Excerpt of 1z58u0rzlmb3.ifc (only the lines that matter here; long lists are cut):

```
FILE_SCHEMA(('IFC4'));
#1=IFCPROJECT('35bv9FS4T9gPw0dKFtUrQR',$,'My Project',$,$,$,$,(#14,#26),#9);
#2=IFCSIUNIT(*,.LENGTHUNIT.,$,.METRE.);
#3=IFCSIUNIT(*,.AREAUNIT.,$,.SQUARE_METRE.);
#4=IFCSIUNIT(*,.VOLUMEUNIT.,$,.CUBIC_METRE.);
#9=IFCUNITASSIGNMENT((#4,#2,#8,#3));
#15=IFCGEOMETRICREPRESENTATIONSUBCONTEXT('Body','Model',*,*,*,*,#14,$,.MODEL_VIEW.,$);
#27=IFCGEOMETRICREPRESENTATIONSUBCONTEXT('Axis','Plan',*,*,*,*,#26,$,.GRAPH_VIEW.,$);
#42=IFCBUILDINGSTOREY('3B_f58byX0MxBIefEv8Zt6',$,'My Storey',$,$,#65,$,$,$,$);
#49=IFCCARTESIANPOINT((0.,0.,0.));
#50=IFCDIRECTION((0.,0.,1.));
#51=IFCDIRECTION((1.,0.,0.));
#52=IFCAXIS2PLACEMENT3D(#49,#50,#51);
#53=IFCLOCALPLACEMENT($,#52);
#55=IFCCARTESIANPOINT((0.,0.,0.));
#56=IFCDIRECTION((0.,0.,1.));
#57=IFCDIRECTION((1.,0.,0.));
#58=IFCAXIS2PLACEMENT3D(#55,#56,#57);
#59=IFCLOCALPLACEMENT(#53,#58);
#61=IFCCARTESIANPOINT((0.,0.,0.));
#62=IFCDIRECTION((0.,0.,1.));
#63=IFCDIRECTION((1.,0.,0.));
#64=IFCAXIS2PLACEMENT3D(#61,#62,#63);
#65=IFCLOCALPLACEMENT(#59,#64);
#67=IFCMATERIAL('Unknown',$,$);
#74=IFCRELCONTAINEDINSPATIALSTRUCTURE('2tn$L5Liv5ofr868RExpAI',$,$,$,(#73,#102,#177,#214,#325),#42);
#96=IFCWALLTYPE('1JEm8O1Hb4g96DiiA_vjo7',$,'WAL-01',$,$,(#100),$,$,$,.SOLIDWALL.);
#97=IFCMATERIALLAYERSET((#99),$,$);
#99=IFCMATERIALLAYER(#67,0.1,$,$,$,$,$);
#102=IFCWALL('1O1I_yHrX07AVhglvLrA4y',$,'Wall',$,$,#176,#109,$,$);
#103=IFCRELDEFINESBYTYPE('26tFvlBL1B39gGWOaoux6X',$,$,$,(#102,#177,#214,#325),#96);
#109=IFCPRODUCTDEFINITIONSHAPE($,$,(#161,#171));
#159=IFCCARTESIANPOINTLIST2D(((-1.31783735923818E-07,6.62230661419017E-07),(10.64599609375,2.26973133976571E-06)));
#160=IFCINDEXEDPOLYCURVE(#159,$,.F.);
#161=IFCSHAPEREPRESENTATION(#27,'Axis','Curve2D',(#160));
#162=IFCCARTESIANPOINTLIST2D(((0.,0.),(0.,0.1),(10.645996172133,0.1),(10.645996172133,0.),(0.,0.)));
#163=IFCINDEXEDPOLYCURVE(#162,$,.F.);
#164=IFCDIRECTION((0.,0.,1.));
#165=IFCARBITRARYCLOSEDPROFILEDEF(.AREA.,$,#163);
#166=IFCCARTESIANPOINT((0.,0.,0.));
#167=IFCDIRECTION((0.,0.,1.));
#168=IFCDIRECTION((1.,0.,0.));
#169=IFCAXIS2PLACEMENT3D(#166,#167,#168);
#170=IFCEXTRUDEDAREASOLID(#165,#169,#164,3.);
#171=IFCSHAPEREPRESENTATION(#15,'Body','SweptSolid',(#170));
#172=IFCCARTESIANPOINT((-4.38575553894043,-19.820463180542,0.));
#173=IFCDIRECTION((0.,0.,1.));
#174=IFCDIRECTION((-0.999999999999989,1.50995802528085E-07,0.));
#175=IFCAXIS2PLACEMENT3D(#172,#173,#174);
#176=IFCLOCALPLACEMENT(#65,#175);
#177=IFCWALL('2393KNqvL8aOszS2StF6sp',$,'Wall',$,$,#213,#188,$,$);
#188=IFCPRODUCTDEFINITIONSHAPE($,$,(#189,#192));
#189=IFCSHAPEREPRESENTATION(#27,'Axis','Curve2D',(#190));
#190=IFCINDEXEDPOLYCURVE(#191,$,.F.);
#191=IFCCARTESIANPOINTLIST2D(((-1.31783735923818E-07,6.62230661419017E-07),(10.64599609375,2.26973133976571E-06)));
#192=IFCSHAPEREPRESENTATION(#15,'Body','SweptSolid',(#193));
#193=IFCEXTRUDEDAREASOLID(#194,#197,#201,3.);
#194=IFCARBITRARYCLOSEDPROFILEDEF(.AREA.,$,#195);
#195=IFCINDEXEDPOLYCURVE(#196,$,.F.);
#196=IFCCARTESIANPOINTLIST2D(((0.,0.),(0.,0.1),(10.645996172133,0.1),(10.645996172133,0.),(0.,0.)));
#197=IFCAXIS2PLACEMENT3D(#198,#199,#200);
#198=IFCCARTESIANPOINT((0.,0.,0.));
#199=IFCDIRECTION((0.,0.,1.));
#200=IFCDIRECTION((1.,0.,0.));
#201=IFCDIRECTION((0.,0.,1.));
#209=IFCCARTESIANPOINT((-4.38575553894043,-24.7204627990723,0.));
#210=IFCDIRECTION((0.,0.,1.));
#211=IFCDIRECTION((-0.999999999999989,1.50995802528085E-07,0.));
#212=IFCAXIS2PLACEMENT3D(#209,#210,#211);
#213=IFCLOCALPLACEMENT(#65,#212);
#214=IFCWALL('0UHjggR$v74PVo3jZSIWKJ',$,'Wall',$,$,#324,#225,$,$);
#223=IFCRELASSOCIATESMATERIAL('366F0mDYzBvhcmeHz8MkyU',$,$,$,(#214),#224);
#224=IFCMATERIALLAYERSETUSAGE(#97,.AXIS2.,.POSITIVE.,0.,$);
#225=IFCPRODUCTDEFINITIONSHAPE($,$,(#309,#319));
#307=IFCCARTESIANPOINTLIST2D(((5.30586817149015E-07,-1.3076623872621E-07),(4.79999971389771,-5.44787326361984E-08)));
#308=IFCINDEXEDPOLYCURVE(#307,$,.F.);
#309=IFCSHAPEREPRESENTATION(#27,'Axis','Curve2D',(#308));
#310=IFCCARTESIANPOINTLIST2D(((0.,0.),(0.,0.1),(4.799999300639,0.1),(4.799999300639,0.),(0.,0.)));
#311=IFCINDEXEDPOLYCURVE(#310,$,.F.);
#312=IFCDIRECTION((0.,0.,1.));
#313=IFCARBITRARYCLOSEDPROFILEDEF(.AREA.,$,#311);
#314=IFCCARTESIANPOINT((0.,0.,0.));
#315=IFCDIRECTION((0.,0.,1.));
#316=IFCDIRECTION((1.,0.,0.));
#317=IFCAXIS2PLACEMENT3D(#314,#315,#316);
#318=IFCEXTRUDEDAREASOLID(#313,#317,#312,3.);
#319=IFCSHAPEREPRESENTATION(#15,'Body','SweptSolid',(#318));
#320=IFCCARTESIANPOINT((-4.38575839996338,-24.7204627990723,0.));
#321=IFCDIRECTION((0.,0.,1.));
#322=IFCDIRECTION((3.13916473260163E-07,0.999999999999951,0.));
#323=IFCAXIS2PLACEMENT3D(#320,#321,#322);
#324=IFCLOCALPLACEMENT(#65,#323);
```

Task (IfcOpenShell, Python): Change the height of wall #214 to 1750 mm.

```python
import ifcopenshell
import ifcopenshell.geom
import ifcopenshell.util.representation
import ifcopenshell.util.shape
import ifcopenshell.util.unit

model = ifcopenshell.open("1z58u0rzlmb3.ifc")
unit_scale = ifcopenshell.util.unit.calculate_unit_scale(model)
settings = ifcopenshell.geom.settings()


def volume(element):
    """Net volume in cubic metres, openings subtracted."""
    shape = ifcopenshell.geom.create_shape(settings, element)
    return ifcopenshell.util.shape.get_volume(shape.geometry)


wall = model.by_guid("0UHjggR$v74PVo3jZSIWKJ")
before = volume(wall)

body = ifcopenshell.util.representation.get_representation(wall, "Model", "Body")
solid = body.Items[0]
old_height = solid.Depth
solid.Depth = 1.75 / unit_scale
after = volume(wall)

print(f"height {old_height:g} -> {solid.Depth:g}, volume {before:.3f} -> {after:.3f} m3")

model.write("1z58u0rzlmb3_v2.ifc")
```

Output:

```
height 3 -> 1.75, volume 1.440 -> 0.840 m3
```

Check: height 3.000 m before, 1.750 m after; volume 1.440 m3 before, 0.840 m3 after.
